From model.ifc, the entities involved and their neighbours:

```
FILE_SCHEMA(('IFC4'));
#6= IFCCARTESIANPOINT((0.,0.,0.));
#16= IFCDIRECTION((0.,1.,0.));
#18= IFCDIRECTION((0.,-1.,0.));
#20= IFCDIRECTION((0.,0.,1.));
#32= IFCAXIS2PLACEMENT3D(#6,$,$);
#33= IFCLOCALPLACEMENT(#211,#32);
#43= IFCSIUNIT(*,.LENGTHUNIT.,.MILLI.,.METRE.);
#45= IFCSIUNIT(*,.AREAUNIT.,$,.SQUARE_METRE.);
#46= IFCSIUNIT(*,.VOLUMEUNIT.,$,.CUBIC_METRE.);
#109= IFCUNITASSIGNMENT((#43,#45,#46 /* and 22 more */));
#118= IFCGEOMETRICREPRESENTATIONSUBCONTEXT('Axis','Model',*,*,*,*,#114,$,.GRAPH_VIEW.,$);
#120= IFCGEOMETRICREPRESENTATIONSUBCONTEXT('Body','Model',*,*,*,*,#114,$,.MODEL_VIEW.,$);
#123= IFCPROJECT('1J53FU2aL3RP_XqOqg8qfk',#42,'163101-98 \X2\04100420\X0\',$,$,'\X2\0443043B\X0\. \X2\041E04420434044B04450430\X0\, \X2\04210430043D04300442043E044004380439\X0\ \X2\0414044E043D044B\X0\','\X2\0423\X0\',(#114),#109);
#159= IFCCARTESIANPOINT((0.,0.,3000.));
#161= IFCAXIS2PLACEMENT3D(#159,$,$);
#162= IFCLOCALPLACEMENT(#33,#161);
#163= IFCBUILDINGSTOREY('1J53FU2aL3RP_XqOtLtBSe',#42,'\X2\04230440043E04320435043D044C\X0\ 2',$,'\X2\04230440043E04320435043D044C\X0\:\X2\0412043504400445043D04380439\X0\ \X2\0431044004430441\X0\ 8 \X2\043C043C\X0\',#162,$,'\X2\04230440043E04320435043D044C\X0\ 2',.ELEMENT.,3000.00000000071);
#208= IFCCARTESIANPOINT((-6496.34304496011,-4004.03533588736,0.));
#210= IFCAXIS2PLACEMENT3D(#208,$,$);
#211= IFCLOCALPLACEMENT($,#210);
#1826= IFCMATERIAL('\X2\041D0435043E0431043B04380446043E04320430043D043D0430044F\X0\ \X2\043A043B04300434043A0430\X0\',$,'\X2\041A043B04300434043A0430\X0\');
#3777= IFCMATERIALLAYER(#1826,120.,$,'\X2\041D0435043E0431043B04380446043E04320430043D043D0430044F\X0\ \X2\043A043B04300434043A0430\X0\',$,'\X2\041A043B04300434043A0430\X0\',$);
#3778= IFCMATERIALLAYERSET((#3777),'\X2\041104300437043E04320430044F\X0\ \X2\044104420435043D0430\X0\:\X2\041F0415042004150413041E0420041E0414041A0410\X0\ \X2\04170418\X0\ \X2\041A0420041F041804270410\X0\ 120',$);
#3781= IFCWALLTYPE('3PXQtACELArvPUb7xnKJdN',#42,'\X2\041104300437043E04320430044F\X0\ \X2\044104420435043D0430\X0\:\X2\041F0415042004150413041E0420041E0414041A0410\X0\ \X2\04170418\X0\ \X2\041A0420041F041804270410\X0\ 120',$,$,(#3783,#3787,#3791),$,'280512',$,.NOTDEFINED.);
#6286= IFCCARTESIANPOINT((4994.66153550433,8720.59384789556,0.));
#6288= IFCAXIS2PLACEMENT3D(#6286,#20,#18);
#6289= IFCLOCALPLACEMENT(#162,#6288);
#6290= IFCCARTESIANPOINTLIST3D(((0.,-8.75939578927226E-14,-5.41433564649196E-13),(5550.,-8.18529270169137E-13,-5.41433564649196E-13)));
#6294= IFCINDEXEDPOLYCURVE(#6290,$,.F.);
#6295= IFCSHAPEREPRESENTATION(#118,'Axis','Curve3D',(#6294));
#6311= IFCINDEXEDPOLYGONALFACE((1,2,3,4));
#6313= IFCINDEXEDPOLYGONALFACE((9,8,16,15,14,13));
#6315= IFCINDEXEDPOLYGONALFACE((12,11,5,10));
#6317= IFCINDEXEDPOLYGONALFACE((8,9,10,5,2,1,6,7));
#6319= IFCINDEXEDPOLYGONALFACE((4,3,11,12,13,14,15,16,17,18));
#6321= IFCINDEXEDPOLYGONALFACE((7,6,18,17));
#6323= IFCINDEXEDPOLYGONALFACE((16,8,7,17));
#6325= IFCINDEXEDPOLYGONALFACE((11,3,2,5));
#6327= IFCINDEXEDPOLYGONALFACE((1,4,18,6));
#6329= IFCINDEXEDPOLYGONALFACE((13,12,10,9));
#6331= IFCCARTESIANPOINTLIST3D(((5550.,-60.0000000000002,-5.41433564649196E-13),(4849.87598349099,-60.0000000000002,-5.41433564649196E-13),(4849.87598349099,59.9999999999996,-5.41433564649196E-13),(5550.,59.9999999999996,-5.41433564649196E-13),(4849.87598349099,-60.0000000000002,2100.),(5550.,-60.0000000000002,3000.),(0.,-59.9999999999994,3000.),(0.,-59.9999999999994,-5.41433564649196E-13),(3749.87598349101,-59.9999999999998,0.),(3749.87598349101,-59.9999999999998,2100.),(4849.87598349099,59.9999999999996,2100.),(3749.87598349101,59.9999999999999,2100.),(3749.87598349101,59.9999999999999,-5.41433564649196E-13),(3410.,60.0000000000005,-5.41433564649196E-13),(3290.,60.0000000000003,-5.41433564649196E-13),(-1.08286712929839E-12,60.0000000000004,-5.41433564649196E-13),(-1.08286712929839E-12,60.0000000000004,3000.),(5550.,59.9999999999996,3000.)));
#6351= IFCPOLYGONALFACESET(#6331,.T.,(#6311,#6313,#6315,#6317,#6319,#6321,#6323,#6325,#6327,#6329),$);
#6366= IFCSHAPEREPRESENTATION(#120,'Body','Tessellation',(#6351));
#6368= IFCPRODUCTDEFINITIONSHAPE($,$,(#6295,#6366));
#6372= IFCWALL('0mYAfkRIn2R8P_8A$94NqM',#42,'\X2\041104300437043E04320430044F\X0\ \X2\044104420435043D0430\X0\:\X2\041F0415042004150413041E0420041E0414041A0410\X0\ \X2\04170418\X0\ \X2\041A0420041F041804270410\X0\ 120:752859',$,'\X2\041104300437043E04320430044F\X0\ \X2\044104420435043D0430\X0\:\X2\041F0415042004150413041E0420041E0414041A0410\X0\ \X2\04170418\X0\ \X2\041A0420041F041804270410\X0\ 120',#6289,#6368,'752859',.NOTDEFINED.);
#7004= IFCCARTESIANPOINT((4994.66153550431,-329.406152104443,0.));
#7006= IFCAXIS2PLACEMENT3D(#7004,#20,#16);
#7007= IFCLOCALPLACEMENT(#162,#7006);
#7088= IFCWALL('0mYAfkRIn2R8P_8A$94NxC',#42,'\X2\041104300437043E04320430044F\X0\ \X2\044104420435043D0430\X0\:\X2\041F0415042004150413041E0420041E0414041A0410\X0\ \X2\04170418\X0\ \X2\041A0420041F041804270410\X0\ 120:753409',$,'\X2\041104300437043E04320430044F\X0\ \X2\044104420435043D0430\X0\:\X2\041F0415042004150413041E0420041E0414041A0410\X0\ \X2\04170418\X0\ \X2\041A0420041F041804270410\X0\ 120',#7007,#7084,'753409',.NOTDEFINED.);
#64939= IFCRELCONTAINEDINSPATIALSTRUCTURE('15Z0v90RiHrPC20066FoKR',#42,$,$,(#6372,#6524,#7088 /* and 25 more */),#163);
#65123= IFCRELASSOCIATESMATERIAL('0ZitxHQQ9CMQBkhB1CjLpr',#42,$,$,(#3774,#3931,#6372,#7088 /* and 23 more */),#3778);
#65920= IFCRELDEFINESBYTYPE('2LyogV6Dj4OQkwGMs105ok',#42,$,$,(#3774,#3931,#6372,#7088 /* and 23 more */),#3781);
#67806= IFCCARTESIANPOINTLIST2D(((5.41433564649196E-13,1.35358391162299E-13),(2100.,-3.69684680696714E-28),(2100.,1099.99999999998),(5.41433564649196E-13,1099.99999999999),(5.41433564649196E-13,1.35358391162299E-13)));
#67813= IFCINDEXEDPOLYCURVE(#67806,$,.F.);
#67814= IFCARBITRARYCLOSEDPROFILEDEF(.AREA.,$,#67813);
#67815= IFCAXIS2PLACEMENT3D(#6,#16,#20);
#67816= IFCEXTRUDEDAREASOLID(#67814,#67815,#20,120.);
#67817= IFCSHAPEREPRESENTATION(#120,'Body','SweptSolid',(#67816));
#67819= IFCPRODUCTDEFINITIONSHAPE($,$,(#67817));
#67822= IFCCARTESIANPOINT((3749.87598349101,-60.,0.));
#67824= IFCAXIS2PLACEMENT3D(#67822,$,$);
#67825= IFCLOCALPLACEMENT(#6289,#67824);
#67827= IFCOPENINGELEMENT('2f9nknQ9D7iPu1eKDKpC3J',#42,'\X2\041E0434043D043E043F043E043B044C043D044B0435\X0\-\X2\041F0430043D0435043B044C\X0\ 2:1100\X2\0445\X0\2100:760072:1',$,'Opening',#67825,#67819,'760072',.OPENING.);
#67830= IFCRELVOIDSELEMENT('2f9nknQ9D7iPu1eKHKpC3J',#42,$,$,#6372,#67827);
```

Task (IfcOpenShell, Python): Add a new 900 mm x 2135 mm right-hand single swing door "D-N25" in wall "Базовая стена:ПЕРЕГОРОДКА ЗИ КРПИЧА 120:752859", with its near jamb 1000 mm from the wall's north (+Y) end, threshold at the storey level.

```python
import numpy as np
import ifcopenshell
import ifcopenshell.api.feature
import ifcopenshell.api.geometry
import ifcopenshell.api.root
import ifcopenshell.api.spatial
import ifcopenshell.geom
import ifcopenshell.util.element
import ifcopenshell.util.placement
import ifcopenshell.util.representation
import ifcopenshell.util.shape
import ifcopenshell.util.unit

model = ifcopenshell.open("model.ifc")
unit_scale = ifcopenshell.util.unit.calculate_unit_scale(model)
settings = ifcopenshell.geom.settings()


def volume(element):
    """Net volume in cubic metres, openings subtracted."""
    shape = ifcopenshell.geom.create_shape(settings, element)
    return ifcopenshell.util.shape.get_volume(shape.geometry)


wall = model.by_id(6372)
storey = ifcopenshell.util.element.get_container(wall, ifc_class="IfcBuildingStorey")
context = ifcopenshell.util.representation.get_context(model, "Model", "Body", "MODEL_VIEW")
before = volume(wall)

width, height, from_end, sill = 0.9, 2.135, 1, 0.0  # metres

# The wall runs along its own X axis, and the end named is its -X end.
wall_shape = ifcopenshell.geom.create_shape(settings, wall)
x, y, z = ifcopenshell.util.shape.get_vertices(wall_shape.geometry).T
start = x.min() + from_end
face, thickness = float(y.min()), float(y.max() - y.min())
wall_matrix = ifcopenshell.util.placement.get_local_placement(wall.ObjectPlacement)
level = ifcopenshell.util.placement.get_local_placement(storey.ObjectPlacement)[2, 3]


def in_wall(x, y):
    """Placement at x, y metres in the wall's axes, at sill height."""
    matrix = wall_matrix.copy()
    matrix[:, 3] = wall_matrix @ np.array([x / unit_scale, y / unit_scale, 0.0, 1.0])
    matrix[2, 3] = level + sill / unit_scale
    return matrix


# Opening: a box that overshoots both wall faces by 50 mm.
opening = ifcopenshell.api.root.create_entity(model, ifc_class="IfcOpeningElement", predefined_type="OPENING")
box = ifcopenshell.api.geometry.add_wall_representation(
    model, context=context, length=width, height=height, thickness=thickness + 0.1
)
ifcopenshell.api.geometry.assign_representation(model, product=opening, representation=box)
ifcopenshell.api.geometry.edit_object_placement(model, product=opening, matrix=in_wall(start, face - 0.05), is_si=False)
ifcopenshell.api.feature.add_feature(model, feature=opening, element=wall)

door = ifcopenshell.api.root.create_entity(model, ifc_class="IfcDoor", name="D-N25", predefined_type="DOOR")
door.OverallWidth, door.OverallHeight = width / unit_scale, height / unit_scale
door.OperationType = "SINGLE_SWING_RIGHT"
body = ifcopenshell.api.geometry.add_door_representation(
    model,
    context=context,
    overall_width=door.OverallWidth,
    overall_height=door.OverallHeight,
    operation_type="SINGLE_SWING_RIGHT",
    lining_properties={"LiningDepth": thickness / unit_scale, "ThresholdDepth": thickness / unit_scale},
)
ifcopenshell.api.geometry.assign_representation(model, product=door, representation=body)
ifcopenshell.api.spatial.assign_container(model, products=[door], relating_structure=storey)
ifcopenshell.api.feature.add_filling(model, opening=opening, element=door)

# The lining spans the wall, so the door starts at the wall face.
ifcopenshell.api.geometry.edit_object_placement(model, product=door, matrix=in_wall(start, face), is_si=False)

after = volume(wall)

print(f"wall volume {before:.3f} -> {after:.3f} m3")

model.write("model_updated.ifc")
```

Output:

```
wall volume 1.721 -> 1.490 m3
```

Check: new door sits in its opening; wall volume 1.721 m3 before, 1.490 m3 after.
